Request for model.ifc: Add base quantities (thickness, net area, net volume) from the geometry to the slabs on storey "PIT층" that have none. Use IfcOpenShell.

First a look at what the model holds.

```python
import ifcopenshell
import ifcopenshell.util.element
import ifcopenshell.util.unit

model = ifcopenshell.open("model.ifc")
print(model.schema)
for unit_type in ("LENGTHUNIT", "AREAUNIT", "VOLUMEUNIT"):
    print(unit_type, ifcopenshell.util.unit.calculate_unit_scale(model, unit_type))
storey = next(s for s in model.by_type("IfcBuildingStorey") if s.Name == "PIT층")
slabs = [e for e in ifcopenshell.util.element.get_decomposition(storey) if e.is_a("IfcSlab")]
for e in sorted(slabs, key=lambda e: e.id()):
    print(e.id(), e.is_a(), e.Name, list(ifcopenshell.util.element.get_psets(e, qtos_only=True)), sep=" | ")
```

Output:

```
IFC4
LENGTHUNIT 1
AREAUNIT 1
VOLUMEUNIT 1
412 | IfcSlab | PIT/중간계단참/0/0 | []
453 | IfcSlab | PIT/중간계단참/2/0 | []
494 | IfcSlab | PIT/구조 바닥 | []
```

```python
import ifcopenshell
import ifcopenshell.api.pset
import ifcopenshell.geom
import ifcopenshell.util.element
import ifcopenshell.util.shape
import ifcopenshell.util.unit

model = ifcopenshell.open("model.ifc")
unit_scale = ifcopenshell.util.unit.calculate_unit_scale(model)
area_scale = ifcopenshell.util.unit.calculate_unit_scale(model, "AREAUNIT")
volume_scale = ifcopenshell.util.unit.calculate_unit_scale(model, "VOLUMEUNIT")
settings = ifcopenshell.geom.settings()

storey = next(s for s in model.by_type("IfcBuildingStorey") if s.Name == "PIT층")
slabs = [e for e in ifcopenshell.util.element.get_decomposition(storey) if e.is_a("IfcSlab")]

for e in sorted(slabs, key=lambda e: e.id()):
    if ifcopenshell.util.element.get_psets(e, qtos_only=True, should_inherit=False):
        continue
    # Geometry comes back in metres, in the element's own axes.
    shape = ifcopenshell.geom.create_shape(settings, e)
    values = {
        "Width": ifcopenshell.util.shape.get_z(shape.geometry) / unit_scale,
        "NetArea": ifcopenshell.util.shape.get_footprint_area(shape.geometry) / area_scale,
        "NetVolume": ifcopenshell.util.shape.get_volume(shape.geometry) / volume_scale,
    }
    qto = ifcopenshell.api.pset.add_qto(model, product=e, name="Qto_SlabBaseQuantities")
    ifcopenshell.api.pset.edit_qto(model, qto=qto, properties=values)
    print(e.id(), {k: round(v, 3) for k, v in values.items()})

model.write("model-out.ifc")
```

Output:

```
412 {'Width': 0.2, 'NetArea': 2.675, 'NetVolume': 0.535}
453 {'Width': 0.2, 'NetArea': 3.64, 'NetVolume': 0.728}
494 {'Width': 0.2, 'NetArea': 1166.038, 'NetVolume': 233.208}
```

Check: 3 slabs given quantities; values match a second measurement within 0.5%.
